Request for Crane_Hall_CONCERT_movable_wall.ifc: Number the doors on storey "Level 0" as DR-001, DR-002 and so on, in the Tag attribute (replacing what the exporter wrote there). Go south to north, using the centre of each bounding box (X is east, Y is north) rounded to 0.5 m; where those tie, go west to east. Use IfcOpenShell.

First a look at what the model holds.

```python
import ifcopenshell
import ifcopenshell.util.element
import ifcopenshell.util.placement

model = ifcopenshell.open("Crane_Hall_CONCERT_movable_wall.ifc")
print(model.schema)
storey = next(s for s in model.by_type("IfcBuildingStorey") if s.Name == "Level 0")
doors = [e for e in ifcopenshell.util.element.get_decomposition(storey) if e.is_a("IfcDoor")]
for e in sorted(doors, key=lambda e: e.id()):
    origin = ifcopenshell.util.placement.get_local_placement(e.ObjectPlacement)[:3, 3]
    print(e.id(), e.Tag, e.Name, origin.round(2) + 0.0, sep=" | ")
```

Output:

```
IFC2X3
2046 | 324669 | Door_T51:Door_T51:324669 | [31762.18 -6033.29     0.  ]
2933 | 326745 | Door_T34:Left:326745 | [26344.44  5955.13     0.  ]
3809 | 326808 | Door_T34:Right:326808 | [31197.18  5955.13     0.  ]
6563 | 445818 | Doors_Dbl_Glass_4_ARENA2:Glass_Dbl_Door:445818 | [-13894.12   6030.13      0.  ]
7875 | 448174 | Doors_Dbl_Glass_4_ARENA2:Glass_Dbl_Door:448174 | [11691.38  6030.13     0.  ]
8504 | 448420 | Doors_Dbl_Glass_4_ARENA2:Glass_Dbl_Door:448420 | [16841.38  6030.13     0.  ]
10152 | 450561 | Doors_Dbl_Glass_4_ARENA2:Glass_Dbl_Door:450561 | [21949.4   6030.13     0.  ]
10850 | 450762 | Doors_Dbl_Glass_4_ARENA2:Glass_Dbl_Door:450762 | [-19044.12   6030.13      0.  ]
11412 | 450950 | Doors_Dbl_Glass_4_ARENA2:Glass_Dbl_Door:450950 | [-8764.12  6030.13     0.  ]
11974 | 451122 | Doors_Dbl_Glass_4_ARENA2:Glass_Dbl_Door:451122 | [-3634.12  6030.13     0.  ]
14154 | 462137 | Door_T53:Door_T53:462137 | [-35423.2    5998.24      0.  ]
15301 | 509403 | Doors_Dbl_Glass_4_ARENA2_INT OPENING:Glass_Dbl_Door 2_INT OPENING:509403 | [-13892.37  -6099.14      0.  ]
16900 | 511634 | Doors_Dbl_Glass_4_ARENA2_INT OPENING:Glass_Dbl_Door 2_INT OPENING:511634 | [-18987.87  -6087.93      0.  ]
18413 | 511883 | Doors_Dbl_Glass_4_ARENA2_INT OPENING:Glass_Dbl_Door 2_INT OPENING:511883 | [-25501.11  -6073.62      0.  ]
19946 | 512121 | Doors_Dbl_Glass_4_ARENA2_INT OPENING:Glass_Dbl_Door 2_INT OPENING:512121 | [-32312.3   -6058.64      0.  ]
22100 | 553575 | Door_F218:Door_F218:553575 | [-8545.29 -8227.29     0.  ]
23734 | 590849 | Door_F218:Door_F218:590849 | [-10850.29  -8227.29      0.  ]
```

```python
import ifcopenshell
import ifcopenshell.geom
import ifcopenshell.util.element
import ifcopenshell.util.shape

model = ifcopenshell.open("Crane_Hall_CONCERT_movable_wall.ifc")
settings = ifcopenshell.geom.settings()
settings.set("use-world-coords", True)


def centre(element):
    shape = ifcopenshell.geom.create_shape(settings, element)
    return ifcopenshell.util.shape.get_bbox_centroid(shape.geometry)


storey = next(s for s in model.by_type("IfcBuildingStorey") if s.Name == "Level 0")
doors = [e for e in ifcopenshell.util.element.get_decomposition(storey) if e.is_a("IfcDoor")]

# Insertion points can sit at a corner or the storey origin, so sort by the geometry (in metres).
centres = {e: centre(e) for e in doors}
doors.sort(key=lambda e: (round(centres[e][1] / 0.5), centres[e][0]))

for i, e in enumerate(doors, start=1):
    number = f"DR-0{i:02d}"
    e.Tag = number
    print(e.id(), number)

model.write("Crane_Hall_CONCERT_movable_wall-out.ifc")
```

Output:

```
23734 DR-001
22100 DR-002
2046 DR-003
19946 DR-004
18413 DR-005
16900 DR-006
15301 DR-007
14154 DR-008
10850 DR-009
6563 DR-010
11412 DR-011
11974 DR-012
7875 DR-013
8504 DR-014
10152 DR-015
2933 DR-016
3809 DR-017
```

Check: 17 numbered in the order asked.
